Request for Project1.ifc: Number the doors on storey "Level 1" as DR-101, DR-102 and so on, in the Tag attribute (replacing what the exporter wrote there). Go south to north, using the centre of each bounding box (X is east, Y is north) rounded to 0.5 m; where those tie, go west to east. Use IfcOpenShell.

First a look at what the model holds.

```python
import ifcopenshell
import ifcopenshell.util.element
import ifcopenshell.util.placement

model = ifcopenshell.open("Project1.ifc")
print(model.schema)
storey = next(s for s in model.by_type("IfcBuildingStorey") if s.Name == "Level 1")
doors = [e for e in ifcopenshell.util.element.get_decomposition(storey) if e.is_a("IfcDoor")]
for e in sorted(doors, key=lambda e: e.id()):
    origin = ifcopenshell.util.placement.get_local_placement(e.ObjectPlacement)[:3, 3]
    print(e.id(), e.Tag, e.Name, origin.round(2) + 0.0, sep=" | ")
```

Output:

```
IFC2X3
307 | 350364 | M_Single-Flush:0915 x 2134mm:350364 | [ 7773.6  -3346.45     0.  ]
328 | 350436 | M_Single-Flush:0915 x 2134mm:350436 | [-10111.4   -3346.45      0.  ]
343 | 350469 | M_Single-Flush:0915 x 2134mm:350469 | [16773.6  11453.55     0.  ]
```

```python
import ifcopenshell
import ifcopenshell.geom
import ifcopenshell.util.element
import ifcopenshell.util.shape

model = ifcopenshell.open("Project1.ifc")
settings = ifcopenshell.geom.settings()
settings.set("use-world-coords", True)


def centre(element):
    shape = ifcopenshell.geom.create_shape(settings, element)
    return ifcopenshell.util.shape.get_bbox_centroid(shape.geometry)


storey = next(s for s in model.by_type("IfcBuildingStorey") if s.Name == "Level 1")
doors = [e for e in ifcopenshell.util.element.get_decomposition(storey) if e.is_a("IfcDoor")]

# Insertion points can sit at a corner or the storey origin, so sort by the geometry (in metres).
centres = {e: centre(e) for e in doors}
doors.sort(key=lambda e: (round(centres[e][1] / 0.5), centres[e][0]))

for i, e in enumerate(doors, start=1):
    number = f"DR-1{i:02d}"
    e.Tag = number
    print(e.id(), number)

model.write("Project1_rev.ifc")
```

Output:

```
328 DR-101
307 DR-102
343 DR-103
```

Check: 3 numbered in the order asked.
